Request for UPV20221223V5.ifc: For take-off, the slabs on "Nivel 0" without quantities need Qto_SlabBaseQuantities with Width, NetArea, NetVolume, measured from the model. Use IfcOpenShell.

First a look at what the model holds.

```python
import ifcopenshell
import ifcopenshell.util.element
import ifcopenshell.util.unit

model = ifcopenshell.open("UPV20221223V5.ifc")
print(model.schema)
for unit_type in ("LENGTHUNIT", "AREAUNIT", "VOLUMEUNIT"):
    print(unit_type, ifcopenshell.util.unit.calculate_unit_scale(model, unit_type))
storey = next(s for s in model.by_type("IfcBuildingStorey") if s.Name == "Nivel 0")
slabs = [e for e in ifcopenshell.util.element.get_decomposition(storey) if e.is_a("IfcSlab")]
for e in sorted(slabs, key=lambda e: e.id()):
    print(e.id(), e.is_a(), e.Name, list(ifcopenshell.util.element.get_psets(e, qtos_only=True)), sep=" | ")
```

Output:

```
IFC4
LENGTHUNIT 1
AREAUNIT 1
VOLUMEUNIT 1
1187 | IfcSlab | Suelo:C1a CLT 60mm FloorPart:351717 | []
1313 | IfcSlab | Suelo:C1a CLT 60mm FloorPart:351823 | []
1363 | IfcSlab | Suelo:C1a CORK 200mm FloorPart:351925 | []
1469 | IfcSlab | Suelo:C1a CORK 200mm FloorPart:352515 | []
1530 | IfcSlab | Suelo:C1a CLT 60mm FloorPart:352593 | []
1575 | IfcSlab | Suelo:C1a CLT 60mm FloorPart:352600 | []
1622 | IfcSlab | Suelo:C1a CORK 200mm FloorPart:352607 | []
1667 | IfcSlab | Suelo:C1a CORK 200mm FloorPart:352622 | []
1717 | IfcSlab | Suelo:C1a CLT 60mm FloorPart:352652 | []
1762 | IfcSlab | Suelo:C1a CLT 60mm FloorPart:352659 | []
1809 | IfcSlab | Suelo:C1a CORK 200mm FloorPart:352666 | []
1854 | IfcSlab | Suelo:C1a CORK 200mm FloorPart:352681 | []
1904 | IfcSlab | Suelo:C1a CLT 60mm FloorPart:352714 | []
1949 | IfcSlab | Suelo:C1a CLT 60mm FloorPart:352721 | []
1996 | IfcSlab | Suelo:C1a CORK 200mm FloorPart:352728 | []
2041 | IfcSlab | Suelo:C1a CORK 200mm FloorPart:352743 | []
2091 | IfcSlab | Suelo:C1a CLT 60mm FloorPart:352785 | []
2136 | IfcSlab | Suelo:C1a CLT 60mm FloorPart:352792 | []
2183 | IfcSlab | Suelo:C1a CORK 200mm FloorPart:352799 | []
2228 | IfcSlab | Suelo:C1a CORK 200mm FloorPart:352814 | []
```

```python
import ifcopenshell
import ifcopenshell.api.pset
import ifcopenshell.geom
import ifcopenshell.util.element
import ifcopenshell.util.shape
import ifcopenshell.util.unit

model = ifcopenshell.open("UPV20221223V5.ifc")
unit_scale = ifcopenshell.util.unit.calculate_unit_scale(model)
area_scale = ifcopenshell.util.unit.calculate_unit_scale(model, "AREAUNIT")
volume_scale = ifcopenshell.util.unit.calculate_unit_scale(model, "VOLUMEUNIT")
settings = ifcopenshell.geom.settings()

storey = next(s for s in model.by_type("IfcBuildingStorey") if s.Name == "Nivel 0")
slabs = [e for e in ifcopenshell.util.element.get_decomposition(storey) if e.is_a("IfcSlab")]

for e in sorted(slabs, key=lambda e: e.id()):
    if ifcopenshell.util.element.get_psets(e, qtos_only=True, should_inherit=False):
        continue
    # Geometry comes back in metres, in the element's own axes.
    shape = ifcopenshell.geom.create_shape(settings, e)
    values = {
        "Width": ifcopenshell.util.shape.get_z(shape.geometry) / unit_scale,
        "NetArea": ifcopenshell.util.shape.get_footprint_area(shape.geometry) / area_scale,
        "NetVolume": ifcopenshell.util.shape.get_volume(shape.geometry) / volume_scale,
    }
    qto = ifcopenshell.api.pset.add_qto(model, product=e, name="Qto_SlabBaseQuantities")
    ifcopenshell.api.pset.edit_qto(model, qto=qto, properties=values)
    print(e.id(), {k: round(v, 3) for k, v in values.items()})

model.write("UPV20221223V5_edited.ifc")
```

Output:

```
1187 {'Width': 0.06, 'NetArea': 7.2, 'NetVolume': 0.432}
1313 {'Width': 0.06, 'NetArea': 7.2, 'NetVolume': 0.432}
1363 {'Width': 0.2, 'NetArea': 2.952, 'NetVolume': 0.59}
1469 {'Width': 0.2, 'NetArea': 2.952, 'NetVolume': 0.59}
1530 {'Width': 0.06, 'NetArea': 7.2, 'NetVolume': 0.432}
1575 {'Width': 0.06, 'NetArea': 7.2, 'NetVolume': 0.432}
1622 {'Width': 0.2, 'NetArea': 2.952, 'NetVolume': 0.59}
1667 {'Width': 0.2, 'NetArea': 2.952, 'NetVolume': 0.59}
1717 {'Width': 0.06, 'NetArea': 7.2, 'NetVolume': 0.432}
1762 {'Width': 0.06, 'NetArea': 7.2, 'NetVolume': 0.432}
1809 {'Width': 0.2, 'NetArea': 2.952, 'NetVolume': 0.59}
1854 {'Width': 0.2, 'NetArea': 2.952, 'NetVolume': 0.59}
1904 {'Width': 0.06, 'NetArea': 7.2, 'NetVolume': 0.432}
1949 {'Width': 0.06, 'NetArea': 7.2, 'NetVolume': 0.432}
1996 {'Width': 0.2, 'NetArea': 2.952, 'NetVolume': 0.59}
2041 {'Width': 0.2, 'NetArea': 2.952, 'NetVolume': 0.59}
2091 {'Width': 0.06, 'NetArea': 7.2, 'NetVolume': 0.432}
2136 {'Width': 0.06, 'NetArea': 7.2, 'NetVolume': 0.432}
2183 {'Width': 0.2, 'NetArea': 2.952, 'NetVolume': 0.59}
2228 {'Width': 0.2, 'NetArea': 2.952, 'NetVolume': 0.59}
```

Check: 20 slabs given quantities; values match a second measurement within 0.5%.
